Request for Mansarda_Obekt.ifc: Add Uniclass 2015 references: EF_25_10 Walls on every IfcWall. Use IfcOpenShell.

First a look at what the model holds.

```python
import ifcopenshell

model = ifcopenshell.open("Mansarda_Obekt.ifc")
print(model.schema)
print("classifications:", [c.Name for c in model.by_type("IfcClassification")])
for ifc_class in ("IfcDoor", "IfcRoof", "IfcStair", "IfcWall", "IfcWindow"):
    print(ifc_class, len(model.by_type(ifc_class)))
```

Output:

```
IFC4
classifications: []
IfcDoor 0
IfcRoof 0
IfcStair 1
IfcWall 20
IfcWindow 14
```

```python
import ifcopenshell
import ifcopenshell.api.classification

model = ifcopenshell.open("Mansarda_Obekt.ifc")

system = ifcopenshell.api.classification.add_classification(model, classification="Uniclass 2015")

codes = {
    "IfcWall": ("EF_25_10", "Walls"),
}
for ifc_class, (code, name) in codes.items():
    products = model.by_type(ifc_class)
    ifcopenshell.api.classification.add_reference(
        model, products=products, classification=system, identification=code, name=name
    )
    print(code, len(products))

model.write("Mansarda_Obekt_rev.ifc")
```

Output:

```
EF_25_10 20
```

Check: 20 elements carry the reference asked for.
